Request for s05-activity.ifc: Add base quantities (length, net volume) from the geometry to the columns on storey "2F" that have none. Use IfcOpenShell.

First a look at what the model holds.

```python
import ifcopenshell
import ifcopenshell.util.element
import ifcopenshell.util.unit

model = ifcopenshell.open("s05-activity.ifc")
print(model.schema)
for unit_type in ("LENGTHUNIT", "AREAUNIT", "VOLUMEUNIT"):
    print(unit_type, ifcopenshell.util.unit.calculate_unit_scale(model, unit_type))
storey = next(s for s in model.by_type("IfcBuildingStorey") if s.Name == "2F")
columns = [e for e in ifcopenshell.util.element.get_decomposition(storey) if e.is_a("IfcColumn")]
for e in sorted(columns, key=lambda e: e.id()):
    print(e.id(), e.is_a(), e.Name, list(ifcopenshell.util.element.get_psets(e, qtos_only=True)), sep=" | ")
```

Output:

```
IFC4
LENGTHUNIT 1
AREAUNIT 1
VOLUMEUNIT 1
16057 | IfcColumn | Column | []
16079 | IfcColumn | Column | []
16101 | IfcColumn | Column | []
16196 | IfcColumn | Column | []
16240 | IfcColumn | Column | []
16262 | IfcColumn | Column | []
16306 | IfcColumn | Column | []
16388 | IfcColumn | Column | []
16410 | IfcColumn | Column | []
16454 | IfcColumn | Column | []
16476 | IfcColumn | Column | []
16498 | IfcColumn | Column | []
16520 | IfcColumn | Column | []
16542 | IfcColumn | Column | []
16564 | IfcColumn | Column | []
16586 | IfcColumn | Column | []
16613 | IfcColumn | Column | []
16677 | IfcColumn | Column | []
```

```python
import ifcopenshell
import ifcopenshell.api.pset
import ifcopenshell.geom
import ifcopenshell.util.element
import ifcopenshell.util.shape
import ifcopenshell.util.unit

model = ifcopenshell.open("s05-activity.ifc")
unit_scale = ifcopenshell.util.unit.calculate_unit_scale(model)
volume_scale = ifcopenshell.util.unit.calculate_unit_scale(model, "VOLUMEUNIT")
settings = ifcopenshell.geom.settings()

storey = next(s for s in model.by_type("IfcBuildingStorey") if s.Name == "2F")
columns = [e for e in ifcopenshell.util.element.get_decomposition(storey) if e.is_a("IfcColumn")]

for e in sorted(columns, key=lambda e: e.id()):
    if ifcopenshell.util.element.get_psets(e, qtos_only=True, should_inherit=False):
        continue
    # Geometry comes back in metres, in the element's own axes.
    shape = ifcopenshell.geom.create_shape(settings, e)
    values = {
        "Length": ifcopenshell.util.shape.get_z(shape.geometry) / unit_scale,
        "NetVolume": ifcopenshell.util.shape.get_volume(shape.geometry) / volume_scale,
    }
    qto = ifcopenshell.api.pset.add_qto(model, product=e, name="Qto_ColumnBaseQuantities")
    ifcopenshell.api.pset.edit_qto(model, qto=qto, properties=values)
    print(e.id(), {k: round(v, 3) for k, v in values.items()})

model.write("s05-activity_rev.ifc")
```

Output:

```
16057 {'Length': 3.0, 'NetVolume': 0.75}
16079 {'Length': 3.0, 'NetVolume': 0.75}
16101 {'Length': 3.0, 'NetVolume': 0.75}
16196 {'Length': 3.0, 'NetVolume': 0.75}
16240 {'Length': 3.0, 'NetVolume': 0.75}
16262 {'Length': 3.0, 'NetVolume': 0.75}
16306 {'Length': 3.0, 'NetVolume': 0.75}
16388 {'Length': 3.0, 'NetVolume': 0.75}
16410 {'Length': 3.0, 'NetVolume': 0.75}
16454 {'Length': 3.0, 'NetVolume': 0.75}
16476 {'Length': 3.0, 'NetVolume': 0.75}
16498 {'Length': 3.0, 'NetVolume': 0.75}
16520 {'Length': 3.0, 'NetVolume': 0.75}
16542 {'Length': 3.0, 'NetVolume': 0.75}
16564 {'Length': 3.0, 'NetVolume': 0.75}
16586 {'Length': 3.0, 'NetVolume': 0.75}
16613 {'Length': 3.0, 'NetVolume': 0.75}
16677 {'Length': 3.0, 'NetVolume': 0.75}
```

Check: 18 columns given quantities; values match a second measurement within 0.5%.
